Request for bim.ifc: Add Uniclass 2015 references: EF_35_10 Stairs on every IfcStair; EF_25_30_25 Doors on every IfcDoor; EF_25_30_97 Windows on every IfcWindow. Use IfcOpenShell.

First a look at what the model holds.

```python
import ifcopenshell

model = ifcopenshell.open("bim.ifc")
print(model.schema)
print("classifications:", [c.Name for c in model.by_type("IfcClassification")])
for ifc_class in ("IfcDoor", "IfcRoof", "IfcStair", "IfcWall", "IfcWindow"):
    print(ifc_class, len(model.by_type(ifc_class)))
```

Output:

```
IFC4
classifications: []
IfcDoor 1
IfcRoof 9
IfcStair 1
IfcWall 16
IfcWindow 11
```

```python
import ifcopenshell
import ifcopenshell.api.classification

model = ifcopenshell.open("bim.ifc")

system = ifcopenshell.api.classification.add_classification(model, classification="Uniclass 2015")

codes = {
    "IfcStair": ("EF_35_10", "Stairs"),
    "IfcDoor": ("EF_25_30_25", "Doors"),
    "IfcWindow": ("EF_25_30_97", "Windows"),
}
for ifc_class, (code, name) in codes.items():
    products = model.by_type(ifc_class)
    ifcopenshell.api.classification.add_reference(
        model, products=products, classification=system, identification=code, name=name
    )
    print(code, len(products))

model.write("bim-out.ifc")
```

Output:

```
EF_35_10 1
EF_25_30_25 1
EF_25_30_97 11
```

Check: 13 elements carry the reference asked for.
